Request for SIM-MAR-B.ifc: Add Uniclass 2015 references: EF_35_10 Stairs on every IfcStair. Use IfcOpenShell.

First a look at what the model holds.

```python
import ifcopenshell

model = ifcopenshell.open("SIM-MAR-B.ifc")
print(model.schema)
print("classifications:", [c.Name for c in model.by_type("IfcClassification")])
for ifc_class in ("IfcDoor", "IfcRoof", "IfcStair", "IfcWall", "IfcWindow"):
    print(ifc_class, len(model.by_type(ifc_class)))
```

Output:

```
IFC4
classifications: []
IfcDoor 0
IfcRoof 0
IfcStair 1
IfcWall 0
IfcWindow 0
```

```python
import ifcopenshell
import ifcopenshell.api.classification

model = ifcopenshell.open("SIM-MAR-B.ifc")

system = ifcopenshell.api.classification.add_classification(model, classification="Uniclass 2015")

codes = {
    "IfcStair": ("EF_35_10", "Stairs"),
}
for ifc_class, (code, name) in codes.items():
    products = model.by_type(ifc_class)
    ifcopenshell.api.classification.add_reference(
        model, products=products, classification=system, identification=code, name=name
    )
    print(code, len(products))

model.write("SIM-MAR-B-out.ifc")
```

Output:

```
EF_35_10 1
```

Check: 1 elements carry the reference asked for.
